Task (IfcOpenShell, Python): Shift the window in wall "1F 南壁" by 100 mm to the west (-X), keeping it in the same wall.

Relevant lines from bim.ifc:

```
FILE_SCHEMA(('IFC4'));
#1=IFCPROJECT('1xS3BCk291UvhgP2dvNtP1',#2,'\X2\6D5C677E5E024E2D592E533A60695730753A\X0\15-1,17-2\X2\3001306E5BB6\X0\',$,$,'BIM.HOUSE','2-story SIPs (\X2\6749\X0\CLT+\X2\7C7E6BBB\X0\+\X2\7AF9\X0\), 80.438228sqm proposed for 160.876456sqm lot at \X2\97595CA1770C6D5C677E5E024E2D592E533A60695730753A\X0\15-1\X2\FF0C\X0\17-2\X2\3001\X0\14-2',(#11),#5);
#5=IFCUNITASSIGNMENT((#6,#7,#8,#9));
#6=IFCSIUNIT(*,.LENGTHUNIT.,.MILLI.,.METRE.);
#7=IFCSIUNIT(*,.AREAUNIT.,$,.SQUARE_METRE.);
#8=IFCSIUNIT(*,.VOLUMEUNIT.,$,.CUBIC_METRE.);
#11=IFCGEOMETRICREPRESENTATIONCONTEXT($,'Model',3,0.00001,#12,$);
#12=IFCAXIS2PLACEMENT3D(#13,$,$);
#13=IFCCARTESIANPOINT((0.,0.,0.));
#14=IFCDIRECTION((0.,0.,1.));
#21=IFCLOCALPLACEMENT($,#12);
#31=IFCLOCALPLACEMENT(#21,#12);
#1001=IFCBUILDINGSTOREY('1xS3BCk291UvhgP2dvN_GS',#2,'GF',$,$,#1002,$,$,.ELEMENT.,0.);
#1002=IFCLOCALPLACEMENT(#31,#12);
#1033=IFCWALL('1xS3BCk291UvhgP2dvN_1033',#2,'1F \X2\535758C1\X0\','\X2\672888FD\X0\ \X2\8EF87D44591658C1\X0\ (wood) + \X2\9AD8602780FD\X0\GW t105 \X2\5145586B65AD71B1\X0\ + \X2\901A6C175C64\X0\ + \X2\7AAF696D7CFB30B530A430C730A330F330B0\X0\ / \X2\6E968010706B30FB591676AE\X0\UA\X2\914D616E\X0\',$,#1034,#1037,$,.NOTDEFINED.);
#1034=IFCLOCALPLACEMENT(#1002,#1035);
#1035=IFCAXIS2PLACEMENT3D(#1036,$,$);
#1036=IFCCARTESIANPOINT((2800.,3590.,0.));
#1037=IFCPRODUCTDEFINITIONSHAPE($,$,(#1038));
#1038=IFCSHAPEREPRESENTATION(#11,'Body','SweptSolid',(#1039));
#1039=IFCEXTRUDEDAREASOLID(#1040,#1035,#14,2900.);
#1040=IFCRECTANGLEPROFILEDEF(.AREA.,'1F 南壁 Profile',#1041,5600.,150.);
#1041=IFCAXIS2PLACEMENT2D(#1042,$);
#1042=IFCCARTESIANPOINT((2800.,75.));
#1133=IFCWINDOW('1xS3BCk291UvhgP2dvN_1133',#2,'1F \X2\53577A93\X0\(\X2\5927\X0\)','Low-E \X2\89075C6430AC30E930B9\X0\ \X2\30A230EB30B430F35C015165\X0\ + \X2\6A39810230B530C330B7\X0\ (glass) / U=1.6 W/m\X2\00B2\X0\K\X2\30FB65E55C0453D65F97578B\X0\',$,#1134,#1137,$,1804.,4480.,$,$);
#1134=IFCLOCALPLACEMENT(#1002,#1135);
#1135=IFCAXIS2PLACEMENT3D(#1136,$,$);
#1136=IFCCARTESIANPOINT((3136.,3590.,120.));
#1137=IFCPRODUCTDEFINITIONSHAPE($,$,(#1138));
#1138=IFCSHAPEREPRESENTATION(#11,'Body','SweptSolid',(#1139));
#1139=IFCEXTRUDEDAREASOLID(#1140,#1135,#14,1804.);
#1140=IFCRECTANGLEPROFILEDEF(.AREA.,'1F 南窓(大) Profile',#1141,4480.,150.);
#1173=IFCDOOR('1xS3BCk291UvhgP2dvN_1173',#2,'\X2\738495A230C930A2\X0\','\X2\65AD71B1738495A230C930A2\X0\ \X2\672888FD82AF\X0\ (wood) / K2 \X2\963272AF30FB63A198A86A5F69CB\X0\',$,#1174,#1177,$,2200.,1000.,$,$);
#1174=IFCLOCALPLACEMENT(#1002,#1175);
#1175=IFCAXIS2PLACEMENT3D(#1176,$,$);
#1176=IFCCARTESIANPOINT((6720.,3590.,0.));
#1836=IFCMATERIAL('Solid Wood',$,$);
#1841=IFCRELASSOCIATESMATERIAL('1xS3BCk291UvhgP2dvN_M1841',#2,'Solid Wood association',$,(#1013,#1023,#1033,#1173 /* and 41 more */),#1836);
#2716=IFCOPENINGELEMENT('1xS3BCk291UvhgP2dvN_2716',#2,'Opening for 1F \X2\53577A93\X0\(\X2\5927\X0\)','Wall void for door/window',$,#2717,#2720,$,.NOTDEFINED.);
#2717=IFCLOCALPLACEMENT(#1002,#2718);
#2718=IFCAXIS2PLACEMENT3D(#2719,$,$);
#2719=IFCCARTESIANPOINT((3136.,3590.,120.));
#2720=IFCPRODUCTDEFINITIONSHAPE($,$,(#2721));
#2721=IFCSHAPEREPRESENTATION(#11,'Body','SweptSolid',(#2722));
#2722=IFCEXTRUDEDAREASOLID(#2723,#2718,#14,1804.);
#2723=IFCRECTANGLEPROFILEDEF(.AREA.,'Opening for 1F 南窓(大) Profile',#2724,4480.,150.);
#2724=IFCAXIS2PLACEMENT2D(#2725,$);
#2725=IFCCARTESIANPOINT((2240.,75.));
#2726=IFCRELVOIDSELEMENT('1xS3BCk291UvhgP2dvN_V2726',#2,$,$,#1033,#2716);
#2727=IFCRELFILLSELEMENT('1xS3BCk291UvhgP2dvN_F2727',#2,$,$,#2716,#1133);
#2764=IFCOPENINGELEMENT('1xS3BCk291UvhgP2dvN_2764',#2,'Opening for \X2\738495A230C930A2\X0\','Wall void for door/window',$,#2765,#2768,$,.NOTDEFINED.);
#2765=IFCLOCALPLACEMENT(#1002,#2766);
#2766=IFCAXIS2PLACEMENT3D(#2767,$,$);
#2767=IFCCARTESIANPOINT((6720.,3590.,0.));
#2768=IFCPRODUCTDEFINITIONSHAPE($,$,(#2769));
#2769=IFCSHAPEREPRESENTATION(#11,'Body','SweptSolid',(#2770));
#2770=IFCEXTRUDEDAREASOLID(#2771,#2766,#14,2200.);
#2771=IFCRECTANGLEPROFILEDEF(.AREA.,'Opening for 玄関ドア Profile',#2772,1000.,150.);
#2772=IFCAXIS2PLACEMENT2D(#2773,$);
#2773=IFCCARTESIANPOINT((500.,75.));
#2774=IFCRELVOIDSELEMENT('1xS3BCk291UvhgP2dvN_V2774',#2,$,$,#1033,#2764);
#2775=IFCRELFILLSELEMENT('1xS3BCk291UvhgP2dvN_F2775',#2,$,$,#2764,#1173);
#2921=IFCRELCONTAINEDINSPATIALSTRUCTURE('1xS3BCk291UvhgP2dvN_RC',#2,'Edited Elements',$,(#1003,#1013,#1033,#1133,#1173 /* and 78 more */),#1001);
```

```python
import ifcopenshell
import ifcopenshell.api.geometry
import ifcopenshell.util.placement

model = ifcopenshell.open("bim.ifc")

window = model.by_id(1133)
opening = window.FillsVoids[0].RelatingOpeningElement
wall = opening.VoidsElements[0].RelatingBuildingElement

wall_matrix = ifcopenshell.util.placement.get_local_placement(wall.ObjectPlacement)
shift = wall_matrix[:3, 0] * -100.0
before = ifcopenshell.util.placement.get_local_placement(window.ObjectPlacement)[:3, 3].copy()

# The window is not placed relative to its opening, so move both.
for product in (opening, window):
    matrix = ifcopenshell.util.placement.get_local_placement(product.ObjectPlacement)
    matrix[:3, 3] += shift
    ifcopenshell.api.geometry.edit_object_placement(model, product=product, matrix=matrix, is_si=False)

after = ifcopenshell.util.placement.get_local_placement(window.ObjectPlacement)[:3, 3]
print("window moved by", (after - before).round(3) + 0.0)

model.write("bim_v2.ifc")
```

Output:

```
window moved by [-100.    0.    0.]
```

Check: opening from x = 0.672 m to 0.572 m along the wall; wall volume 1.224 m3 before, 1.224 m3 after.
